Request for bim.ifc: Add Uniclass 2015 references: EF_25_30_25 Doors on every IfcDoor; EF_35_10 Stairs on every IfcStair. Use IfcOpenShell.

First a look at what the model holds.

```python
import ifcopenshell

model = ifcopenshell.open("bim.ifc")
print(model.schema)
print("classifications:", [c.Name for c in model.by_type("IfcClassification")])
for ifc_class in ("IfcDoor", "IfcRoof", "IfcStair", "IfcWall", "IfcWindow"):
    print(ifc_class, len(model.by_type(ifc_class)))
```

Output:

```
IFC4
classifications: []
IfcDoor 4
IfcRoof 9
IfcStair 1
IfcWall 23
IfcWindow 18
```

```python
import ifcopenshell
import ifcopenshell.api.classification

model = ifcopenshell.open("bim.ifc")

system = ifcopenshell.api.classification.add_classification(model, classification="Uniclass 2015")

codes = {
    "IfcDoor": ("EF_25_30_25", "Doors"),
    "IfcStair": ("EF_35_10", "Stairs"),
}
for ifc_class, (code, name) in codes.items():
    products = model.by_type(ifc_class)
    ifcopenshell.api.classification.add_reference(
        model, products=products, classification=system, identification=code, name=name
    )
    print(code, len(products))

model.write("bim_v2.ifc")
```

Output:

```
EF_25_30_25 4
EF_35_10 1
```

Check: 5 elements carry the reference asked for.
